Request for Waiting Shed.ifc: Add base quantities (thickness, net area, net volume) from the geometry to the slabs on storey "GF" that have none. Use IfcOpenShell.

First a look at what the model holds.

```python
import ifcopenshell
import ifcopenshell.util.element
import ifcopenshell.util.unit

model = ifcopenshell.open("Waiting Shed.ifc")
print(model.schema)
for unit_type in ("LENGTHUNIT", "AREAUNIT", "VOLUMEUNIT"):
    print(unit_type, ifcopenshell.util.unit.calculate_unit_scale(model, unit_type))
storey = next(s for s in model.by_type("IfcBuildingStorey") if s.Name == "GF")
slabs = [e for e in ifcopenshell.util.element.get_decomposition(storey) if e.is_a("IfcSlab")]
for e in sorted(slabs, key=lambda e: e.id()):
    print(e.id(), e.is_a(), e.Name, list(ifcopenshell.util.element.get_psets(e, qtos_only=True)), sep=" | ")
```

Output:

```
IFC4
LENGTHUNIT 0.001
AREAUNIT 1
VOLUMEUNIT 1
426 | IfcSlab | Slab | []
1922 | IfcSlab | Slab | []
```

```python
import ifcopenshell
import ifcopenshell.api.pset
import ifcopenshell.geom
import ifcopenshell.util.element
import ifcopenshell.util.shape
import ifcopenshell.util.unit

model = ifcopenshell.open("Waiting Shed.ifc")
unit_scale = ifcopenshell.util.unit.calculate_unit_scale(model)
area_scale = ifcopenshell.util.unit.calculate_unit_scale(model, "AREAUNIT")
volume_scale = ifcopenshell.util.unit.calculate_unit_scale(model, "VOLUMEUNIT")
settings = ifcopenshell.geom.settings()

storey = next(s for s in model.by_type("IfcBuildingStorey") if s.Name == "GF")
slabs = [e for e in ifcopenshell.util.element.get_decomposition(storey) if e.is_a("IfcSlab")]

for e in sorted(slabs, key=lambda e: e.id()):
    if ifcopenshell.util.element.get_psets(e, qtos_only=True, should_inherit=False):
        continue
    # Geometry comes back in metres, in the element's own axes.
    shape = ifcopenshell.geom.create_shape(settings, e)
    values = {
        "Width": ifcopenshell.util.shape.get_z(shape.geometry) / unit_scale,
        "NetArea": ifcopenshell.util.shape.get_footprint_area(shape.geometry) / area_scale,
        "NetVolume": ifcopenshell.util.shape.get_volume(shape.geometry) / volume_scale,
    }
    qto = ifcopenshell.api.pset.add_qto(model, product=e, name="Qto_SlabBaseQuantities")
    ifcopenshell.api.pset.edit_qto(model, qto=qto, properties=values)
    print(e.id(), {k: round(v, 3) for k, v in values.items()})

model.write("Waiting Shed-out.ifc")
```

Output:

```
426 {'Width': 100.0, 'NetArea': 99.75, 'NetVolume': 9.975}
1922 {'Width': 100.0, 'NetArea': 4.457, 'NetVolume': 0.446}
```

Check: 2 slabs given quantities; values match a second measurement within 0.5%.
